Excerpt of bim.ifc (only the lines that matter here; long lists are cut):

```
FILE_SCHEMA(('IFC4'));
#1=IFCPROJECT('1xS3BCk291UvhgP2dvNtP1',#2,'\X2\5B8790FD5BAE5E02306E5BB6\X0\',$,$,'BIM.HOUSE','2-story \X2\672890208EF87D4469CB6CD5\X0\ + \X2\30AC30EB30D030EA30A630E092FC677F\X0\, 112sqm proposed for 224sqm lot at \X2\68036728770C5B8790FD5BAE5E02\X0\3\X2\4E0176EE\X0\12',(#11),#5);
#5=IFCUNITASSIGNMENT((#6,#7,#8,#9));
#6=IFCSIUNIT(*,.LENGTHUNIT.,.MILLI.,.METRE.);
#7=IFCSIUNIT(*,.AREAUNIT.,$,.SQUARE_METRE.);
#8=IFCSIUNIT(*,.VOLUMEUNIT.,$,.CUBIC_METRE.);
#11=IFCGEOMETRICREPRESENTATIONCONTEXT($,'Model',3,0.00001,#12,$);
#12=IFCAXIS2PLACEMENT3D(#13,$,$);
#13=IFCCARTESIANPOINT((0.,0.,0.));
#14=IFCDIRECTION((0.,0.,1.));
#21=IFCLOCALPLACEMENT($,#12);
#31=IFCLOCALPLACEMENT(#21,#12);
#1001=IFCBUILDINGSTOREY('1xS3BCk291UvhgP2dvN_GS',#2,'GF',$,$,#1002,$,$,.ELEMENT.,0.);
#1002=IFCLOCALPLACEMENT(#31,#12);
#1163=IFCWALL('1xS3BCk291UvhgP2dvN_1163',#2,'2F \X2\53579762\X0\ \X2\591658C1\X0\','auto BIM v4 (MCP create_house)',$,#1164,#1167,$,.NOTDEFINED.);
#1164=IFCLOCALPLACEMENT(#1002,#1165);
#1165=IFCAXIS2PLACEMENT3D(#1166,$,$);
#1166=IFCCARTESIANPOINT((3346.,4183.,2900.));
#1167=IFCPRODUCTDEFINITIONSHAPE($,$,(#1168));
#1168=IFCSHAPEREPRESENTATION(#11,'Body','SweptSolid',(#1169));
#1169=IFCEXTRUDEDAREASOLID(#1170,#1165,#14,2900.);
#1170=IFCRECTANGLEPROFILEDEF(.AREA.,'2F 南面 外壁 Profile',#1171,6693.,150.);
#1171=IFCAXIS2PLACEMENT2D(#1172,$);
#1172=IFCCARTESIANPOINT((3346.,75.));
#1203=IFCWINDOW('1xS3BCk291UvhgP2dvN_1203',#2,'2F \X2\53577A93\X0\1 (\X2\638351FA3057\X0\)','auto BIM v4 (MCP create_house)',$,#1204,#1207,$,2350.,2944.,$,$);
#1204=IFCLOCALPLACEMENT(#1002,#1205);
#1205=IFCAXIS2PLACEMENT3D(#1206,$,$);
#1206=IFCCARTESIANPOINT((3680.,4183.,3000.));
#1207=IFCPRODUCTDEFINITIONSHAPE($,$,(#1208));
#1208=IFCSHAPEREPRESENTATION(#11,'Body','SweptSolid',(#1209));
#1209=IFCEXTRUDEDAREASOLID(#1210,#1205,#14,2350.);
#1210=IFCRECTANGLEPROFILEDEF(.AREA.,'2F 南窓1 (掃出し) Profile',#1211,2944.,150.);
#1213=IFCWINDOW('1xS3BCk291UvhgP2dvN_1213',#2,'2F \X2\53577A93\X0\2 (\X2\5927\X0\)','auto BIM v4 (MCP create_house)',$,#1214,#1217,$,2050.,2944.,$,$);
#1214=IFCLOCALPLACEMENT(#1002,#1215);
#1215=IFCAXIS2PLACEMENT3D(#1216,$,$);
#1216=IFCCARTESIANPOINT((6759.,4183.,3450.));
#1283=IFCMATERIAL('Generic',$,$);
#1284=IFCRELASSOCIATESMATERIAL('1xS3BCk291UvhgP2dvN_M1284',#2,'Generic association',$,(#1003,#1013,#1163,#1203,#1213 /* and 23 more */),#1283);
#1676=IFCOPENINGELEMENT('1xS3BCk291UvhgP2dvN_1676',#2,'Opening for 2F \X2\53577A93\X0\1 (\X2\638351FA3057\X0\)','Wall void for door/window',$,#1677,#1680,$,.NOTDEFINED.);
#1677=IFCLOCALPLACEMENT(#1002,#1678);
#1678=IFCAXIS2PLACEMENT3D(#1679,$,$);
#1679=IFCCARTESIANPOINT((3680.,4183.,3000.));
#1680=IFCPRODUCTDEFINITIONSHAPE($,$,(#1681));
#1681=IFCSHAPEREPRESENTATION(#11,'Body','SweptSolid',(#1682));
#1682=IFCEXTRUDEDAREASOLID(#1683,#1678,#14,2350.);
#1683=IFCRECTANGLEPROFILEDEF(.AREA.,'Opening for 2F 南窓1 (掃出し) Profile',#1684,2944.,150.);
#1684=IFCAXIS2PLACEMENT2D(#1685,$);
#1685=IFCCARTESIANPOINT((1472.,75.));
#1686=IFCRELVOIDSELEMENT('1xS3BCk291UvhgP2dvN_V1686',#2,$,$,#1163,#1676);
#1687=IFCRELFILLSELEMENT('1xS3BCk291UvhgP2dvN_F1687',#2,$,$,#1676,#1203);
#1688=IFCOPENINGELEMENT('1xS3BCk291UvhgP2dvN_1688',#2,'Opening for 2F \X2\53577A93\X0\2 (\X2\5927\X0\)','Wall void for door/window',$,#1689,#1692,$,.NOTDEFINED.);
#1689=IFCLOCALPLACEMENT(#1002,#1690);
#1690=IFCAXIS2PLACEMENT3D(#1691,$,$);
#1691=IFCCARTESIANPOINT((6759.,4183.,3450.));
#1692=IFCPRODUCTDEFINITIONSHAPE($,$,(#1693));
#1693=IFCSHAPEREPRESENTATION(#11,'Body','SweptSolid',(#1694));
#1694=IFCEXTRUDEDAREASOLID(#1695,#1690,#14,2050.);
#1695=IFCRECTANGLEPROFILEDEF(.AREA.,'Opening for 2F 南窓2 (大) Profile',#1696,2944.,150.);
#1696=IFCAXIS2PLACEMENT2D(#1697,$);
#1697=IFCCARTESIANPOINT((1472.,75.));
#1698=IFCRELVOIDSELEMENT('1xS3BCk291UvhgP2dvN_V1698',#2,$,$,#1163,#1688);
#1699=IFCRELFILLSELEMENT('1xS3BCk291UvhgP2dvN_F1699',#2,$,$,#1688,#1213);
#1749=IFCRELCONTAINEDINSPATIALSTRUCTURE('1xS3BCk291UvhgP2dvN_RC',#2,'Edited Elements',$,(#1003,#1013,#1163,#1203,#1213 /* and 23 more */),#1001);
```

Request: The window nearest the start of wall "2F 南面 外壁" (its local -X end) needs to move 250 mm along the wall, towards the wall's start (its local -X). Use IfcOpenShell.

```python
import ifcopenshell
import ifcopenshell.api.geometry
import ifcopenshell.util.placement

model = ifcopenshell.open("bim.ifc")

window = model.by_guid("1xS3BCk291UvhgP2dvN_1203")
opening = window.FillsVoids[0].RelatingOpeningElement
wall = opening.VoidsElements[0].RelatingBuildingElement

wall_matrix = ifcopenshell.util.placement.get_local_placement(wall.ObjectPlacement)
shift = wall_matrix[:3, 0] * -250.0
before = ifcopenshell.util.placement.get_local_placement(window.ObjectPlacement)[:3, 3].copy()

# The window is not placed relative to its opening, so move both.
for product in (opening, window):
    matrix = ifcopenshell.util.placement.get_local_placement(product.ObjectPlacement)
    matrix[:3, 3] += shift
    ifcopenshell.api.geometry.edit_object_placement(model, product=product, matrix=matrix, is_si=False)

after = ifcopenshell.util.placement.get_local_placement(window.ObjectPlacement)[:3, 3]
print("window moved by", (after - before).round(3) + 0.0)

model.write("bim_updated.ifc")
```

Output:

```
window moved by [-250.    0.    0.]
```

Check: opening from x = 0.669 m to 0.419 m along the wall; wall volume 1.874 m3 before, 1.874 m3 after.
